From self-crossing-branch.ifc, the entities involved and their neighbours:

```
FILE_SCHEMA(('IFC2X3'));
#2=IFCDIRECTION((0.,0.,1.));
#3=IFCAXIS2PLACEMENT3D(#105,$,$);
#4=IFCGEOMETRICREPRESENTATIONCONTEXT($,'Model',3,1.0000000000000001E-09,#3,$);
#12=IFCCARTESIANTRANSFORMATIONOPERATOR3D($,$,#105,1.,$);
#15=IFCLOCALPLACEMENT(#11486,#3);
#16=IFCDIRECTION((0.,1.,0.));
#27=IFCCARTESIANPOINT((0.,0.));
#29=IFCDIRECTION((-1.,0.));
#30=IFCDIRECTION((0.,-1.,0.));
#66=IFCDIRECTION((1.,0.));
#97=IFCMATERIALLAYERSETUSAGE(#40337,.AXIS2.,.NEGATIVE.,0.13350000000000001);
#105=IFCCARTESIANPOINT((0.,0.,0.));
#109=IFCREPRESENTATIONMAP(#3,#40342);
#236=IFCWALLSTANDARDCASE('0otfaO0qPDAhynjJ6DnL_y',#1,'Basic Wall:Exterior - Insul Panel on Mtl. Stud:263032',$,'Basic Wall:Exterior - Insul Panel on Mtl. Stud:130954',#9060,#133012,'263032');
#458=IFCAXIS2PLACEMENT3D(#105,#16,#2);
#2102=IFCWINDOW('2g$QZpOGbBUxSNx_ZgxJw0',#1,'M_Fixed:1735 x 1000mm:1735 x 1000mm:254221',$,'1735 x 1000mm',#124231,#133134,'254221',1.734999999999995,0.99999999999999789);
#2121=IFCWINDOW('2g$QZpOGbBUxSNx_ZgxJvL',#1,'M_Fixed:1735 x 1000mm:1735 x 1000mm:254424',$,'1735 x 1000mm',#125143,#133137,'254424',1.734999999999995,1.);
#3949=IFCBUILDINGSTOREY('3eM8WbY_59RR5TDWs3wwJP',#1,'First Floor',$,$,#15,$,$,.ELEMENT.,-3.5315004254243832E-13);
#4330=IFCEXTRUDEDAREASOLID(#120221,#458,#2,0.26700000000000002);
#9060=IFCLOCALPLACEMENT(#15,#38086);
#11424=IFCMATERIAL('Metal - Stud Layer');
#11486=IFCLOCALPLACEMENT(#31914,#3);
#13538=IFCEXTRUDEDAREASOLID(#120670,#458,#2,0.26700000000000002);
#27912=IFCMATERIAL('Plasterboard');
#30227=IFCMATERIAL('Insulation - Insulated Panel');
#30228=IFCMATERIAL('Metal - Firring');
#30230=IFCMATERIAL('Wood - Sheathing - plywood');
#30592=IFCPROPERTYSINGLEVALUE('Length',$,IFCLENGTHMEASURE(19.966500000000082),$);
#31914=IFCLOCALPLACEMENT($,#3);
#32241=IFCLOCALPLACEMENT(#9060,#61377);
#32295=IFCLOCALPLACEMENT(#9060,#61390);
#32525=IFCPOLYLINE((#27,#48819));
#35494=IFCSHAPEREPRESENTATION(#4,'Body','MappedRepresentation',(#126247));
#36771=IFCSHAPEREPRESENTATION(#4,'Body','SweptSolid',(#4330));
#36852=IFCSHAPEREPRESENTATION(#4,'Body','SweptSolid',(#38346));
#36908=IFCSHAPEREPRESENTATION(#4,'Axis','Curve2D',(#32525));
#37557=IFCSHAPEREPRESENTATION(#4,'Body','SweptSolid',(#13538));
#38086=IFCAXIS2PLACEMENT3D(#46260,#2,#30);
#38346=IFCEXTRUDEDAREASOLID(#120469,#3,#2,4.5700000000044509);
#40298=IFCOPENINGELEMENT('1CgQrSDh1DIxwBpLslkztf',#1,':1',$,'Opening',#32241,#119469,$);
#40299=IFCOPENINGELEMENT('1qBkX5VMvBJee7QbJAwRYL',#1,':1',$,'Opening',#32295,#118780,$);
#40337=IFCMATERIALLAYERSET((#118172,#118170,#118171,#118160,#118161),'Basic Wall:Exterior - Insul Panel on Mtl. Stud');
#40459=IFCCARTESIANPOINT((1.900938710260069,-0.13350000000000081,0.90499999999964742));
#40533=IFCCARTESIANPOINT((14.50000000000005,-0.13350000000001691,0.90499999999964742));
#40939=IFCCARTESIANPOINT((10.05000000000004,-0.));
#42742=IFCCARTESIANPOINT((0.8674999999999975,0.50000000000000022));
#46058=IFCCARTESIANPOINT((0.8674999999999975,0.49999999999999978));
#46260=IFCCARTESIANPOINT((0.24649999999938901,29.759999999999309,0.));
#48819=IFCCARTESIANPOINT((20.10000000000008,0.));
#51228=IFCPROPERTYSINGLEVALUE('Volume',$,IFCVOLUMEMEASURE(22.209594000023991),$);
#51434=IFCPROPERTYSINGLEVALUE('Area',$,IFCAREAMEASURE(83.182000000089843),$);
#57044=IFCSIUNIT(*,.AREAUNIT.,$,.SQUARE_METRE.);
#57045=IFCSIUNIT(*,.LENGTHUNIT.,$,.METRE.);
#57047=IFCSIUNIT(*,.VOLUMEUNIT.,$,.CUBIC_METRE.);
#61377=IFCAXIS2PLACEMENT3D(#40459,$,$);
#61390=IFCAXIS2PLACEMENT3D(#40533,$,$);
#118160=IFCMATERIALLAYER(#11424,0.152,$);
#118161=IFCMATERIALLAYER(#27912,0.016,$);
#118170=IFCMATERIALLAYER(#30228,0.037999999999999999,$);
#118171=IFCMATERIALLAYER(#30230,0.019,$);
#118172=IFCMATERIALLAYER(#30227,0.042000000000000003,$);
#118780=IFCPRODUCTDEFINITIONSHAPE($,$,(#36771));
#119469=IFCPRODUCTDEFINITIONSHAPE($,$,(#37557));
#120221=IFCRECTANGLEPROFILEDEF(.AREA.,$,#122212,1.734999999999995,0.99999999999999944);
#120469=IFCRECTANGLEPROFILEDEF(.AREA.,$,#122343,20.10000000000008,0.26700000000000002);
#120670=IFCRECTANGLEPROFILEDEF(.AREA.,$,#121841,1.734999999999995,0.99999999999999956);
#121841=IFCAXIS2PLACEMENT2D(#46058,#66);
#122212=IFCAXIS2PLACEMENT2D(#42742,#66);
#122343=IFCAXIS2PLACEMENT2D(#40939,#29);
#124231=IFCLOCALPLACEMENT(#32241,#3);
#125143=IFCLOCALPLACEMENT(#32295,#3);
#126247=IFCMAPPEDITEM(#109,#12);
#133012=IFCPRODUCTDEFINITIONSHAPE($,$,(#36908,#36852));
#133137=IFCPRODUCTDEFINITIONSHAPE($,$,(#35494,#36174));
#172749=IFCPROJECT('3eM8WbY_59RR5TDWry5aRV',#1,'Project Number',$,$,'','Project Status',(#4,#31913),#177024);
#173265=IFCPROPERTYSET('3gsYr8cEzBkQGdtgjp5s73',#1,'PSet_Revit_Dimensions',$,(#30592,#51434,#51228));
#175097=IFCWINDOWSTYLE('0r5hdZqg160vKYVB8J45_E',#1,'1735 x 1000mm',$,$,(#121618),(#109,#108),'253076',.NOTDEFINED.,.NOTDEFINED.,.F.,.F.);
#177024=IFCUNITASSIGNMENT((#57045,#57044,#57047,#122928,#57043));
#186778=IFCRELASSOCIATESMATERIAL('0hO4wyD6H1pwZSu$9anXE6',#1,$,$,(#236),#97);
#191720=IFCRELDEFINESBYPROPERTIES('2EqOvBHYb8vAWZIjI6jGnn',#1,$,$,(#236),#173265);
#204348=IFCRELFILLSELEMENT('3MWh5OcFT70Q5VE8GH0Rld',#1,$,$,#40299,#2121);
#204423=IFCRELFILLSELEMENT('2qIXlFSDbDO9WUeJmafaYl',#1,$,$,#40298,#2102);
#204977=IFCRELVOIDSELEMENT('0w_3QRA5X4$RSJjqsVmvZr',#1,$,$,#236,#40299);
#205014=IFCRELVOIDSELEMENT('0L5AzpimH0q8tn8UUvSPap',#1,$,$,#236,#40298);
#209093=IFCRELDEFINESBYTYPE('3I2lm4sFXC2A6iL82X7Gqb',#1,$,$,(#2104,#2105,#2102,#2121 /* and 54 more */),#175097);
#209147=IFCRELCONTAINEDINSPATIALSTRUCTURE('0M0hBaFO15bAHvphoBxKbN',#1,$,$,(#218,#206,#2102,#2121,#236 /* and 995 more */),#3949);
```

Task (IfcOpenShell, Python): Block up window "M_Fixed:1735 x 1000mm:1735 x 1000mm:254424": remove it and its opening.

```python
import ifcopenshell
import ifcopenshell.api.feature
import ifcopenshell.api.pset
import ifcopenshell.api.root
import ifcopenshell.geom
import ifcopenshell.util.element
import ifcopenshell.util.shape
import ifcopenshell.util.unit

model = ifcopenshell.open("self-crossing-branch.ifc")
area_scale = ifcopenshell.util.unit.calculate_unit_scale(model, "AREAUNIT")
volume_scale = ifcopenshell.util.unit.calculate_unit_scale(model, "VOLUMEUNIT")
settings = ifcopenshell.geom.settings()


def volume(element):
    """Net volume in cubic metres, openings subtracted."""
    shape = ifcopenshell.geom.create_shape(settings, element)
    return ifcopenshell.util.shape.get_volume(shape.geometry)


window = model.by_guid("2g$QZpOGbBUxSNx_ZgxJvL")
opening = window.FillsVoids[0].RelatingOpeningElement
wall = opening.VoidsElements[0].RelatingBuildingElement
before = volume(wall)

ifcopenshell.api.root.remove_product(model, product=window)
ifcopenshell.api.feature.remove_feature(model, feature=opening)

after = volume(wall)
thickness = 0.267  # wall thickness in metres

# Update the wall's stored quantities.
pset = model.by_id(ifcopenshell.util.element.get_pset(wall, "PSet_Revit_Dimensions", should_inherit=False)["id"])
ifcopenshell.api.pset.edit_pset(model, pset=pset, properties={
    "Area": model.create_entity("IfcAreaMeasure", after / thickness / area_scale),
    "Volume": model.create_entity("IfcVolumeMeasure", after / volume_scale),
})

print(f"wall volume {before:.3f} -> {after:.3f} m3")

model.write("self-crossing-branch_v2.ifc")
```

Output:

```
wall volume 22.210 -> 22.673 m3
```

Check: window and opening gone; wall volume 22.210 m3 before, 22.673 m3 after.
